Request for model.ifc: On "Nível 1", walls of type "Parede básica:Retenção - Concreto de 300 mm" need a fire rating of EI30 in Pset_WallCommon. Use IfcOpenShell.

First a look at what the model holds.

```python
import ifcopenshell
import ifcopenshell.util.element

model = ifcopenshell.open("model.ifc")
print(model.schema)
storey = next(s for s in model.by_type("IfcBuildingStorey") if s.Name == "Nível 1")
walls = [e for e in ifcopenshell.util.element.get_decomposition(storey) if e.is_a("IfcWall")]
seen = {}
for e in walls:
    element_type = ifcopenshell.util.element.get_type(e)
    key = (element_type.Name if element_type != e and element_type else None, ifcopenshell.util.element.get_pset(e, "Pset_WallCommon", "FireRating"))
    seen[key] = seen.get(key, 0) + 1
for (name, value), count in sorted(seen.items(), key=str):
    print(count, "x", name, "|", value)
```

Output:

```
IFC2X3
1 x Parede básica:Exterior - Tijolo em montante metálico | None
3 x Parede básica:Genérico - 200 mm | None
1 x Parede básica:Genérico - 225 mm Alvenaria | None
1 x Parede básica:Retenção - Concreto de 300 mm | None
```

```python
import ifcopenshell
import ifcopenshell.api.pset
import ifcopenshell.util.element

model = ifcopenshell.open("model.ifc")

storey = next(s for s in model.by_type("IfcBuildingStorey") if s.Name == "Nível 1")
walls = [e for e in ifcopenshell.util.element.get_decomposition(storey) if e.is_a("IfcWall")]

count = 0
for e in walls:
    element_type = ifcopenshell.util.element.get_type(e)
    if element_type in (None, e) or element_type.Name != "Parede básica:Retenção - Concreto de 300 mm":
        continue
    # add_pset returns the element's existing set when there is one.
    pset = ifcopenshell.api.pset.add_pset(model, product=e, name="Pset_WallCommon")
    ifcopenshell.api.pset.edit_pset(model, pset=pset, properties={"FireRating": "EI30"})
    count += 1

print(count, "walls updated")

model.write("model_edited.ifc")
```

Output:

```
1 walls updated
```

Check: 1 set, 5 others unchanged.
